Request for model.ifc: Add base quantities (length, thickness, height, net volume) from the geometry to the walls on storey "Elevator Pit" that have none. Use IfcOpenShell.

First a look at what the model holds.

```python
import ifcopenshell
import ifcopenshell.util.element
import ifcopenshell.util.unit

model = ifcopenshell.open("model.ifc")
print(model.schema)
for unit_type in ("LENGTHUNIT", "AREAUNIT", "VOLUMEUNIT"):
    print(unit_type, ifcopenshell.util.unit.calculate_unit_scale(model, unit_type))
storey = next(s for s in model.by_type("IfcBuildingStorey") if s.Name == "Elevator Pit")
walls = [e for e in ifcopenshell.util.element.get_decomposition(storey) if e.is_a("IfcWall")]
for e in sorted(walls, key=lambda e: e.id()):
    print(e.id(), e.is_a(), e.Name, list(ifcopenshell.util.element.get_psets(e, qtos_only=True)), sep=" | ")
```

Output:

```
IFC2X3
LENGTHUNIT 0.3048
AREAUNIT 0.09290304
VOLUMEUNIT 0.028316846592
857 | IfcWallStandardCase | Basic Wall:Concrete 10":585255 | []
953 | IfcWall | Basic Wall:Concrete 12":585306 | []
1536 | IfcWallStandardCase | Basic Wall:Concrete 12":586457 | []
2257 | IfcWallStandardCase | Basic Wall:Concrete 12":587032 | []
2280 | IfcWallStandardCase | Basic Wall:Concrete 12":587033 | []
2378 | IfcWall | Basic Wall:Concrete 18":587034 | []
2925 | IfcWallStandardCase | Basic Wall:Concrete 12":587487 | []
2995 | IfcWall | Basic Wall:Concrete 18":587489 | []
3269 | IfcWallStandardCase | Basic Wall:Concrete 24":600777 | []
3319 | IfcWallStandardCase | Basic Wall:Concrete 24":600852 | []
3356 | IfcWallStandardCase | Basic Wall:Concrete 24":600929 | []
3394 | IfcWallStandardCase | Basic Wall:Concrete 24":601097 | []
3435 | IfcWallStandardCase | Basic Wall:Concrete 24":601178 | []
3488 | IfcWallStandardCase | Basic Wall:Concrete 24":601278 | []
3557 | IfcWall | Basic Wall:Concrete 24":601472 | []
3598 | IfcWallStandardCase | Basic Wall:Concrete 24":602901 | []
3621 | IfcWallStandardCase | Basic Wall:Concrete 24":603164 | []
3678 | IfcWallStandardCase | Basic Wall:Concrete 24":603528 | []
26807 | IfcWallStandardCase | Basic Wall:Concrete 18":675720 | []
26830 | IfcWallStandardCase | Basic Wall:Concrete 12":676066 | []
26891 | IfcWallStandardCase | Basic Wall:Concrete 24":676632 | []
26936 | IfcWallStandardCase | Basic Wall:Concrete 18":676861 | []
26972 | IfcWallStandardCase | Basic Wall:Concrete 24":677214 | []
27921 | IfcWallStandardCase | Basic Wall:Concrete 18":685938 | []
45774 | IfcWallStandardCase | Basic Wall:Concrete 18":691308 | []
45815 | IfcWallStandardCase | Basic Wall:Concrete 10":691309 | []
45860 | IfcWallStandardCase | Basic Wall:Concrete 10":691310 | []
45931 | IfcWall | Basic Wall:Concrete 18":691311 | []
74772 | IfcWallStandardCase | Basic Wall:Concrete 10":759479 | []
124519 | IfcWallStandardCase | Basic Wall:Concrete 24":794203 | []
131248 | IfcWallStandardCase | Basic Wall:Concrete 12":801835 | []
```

```python
import ifcopenshell
import ifcopenshell.api.pset
import ifcopenshell.geom
import ifcopenshell.util.element
import ifcopenshell.util.shape
import ifcopenshell.util.unit

model = ifcopenshell.open("model.ifc")
unit_scale = ifcopenshell.util.unit.calculate_unit_scale(model)
volume_scale = ifcopenshell.util.unit.calculate_unit_scale(model, "VOLUMEUNIT")
settings = ifcopenshell.geom.settings()

storey = next(s for s in model.by_type("IfcBuildingStorey") if s.Name == "Elevator Pit")
walls = [e for e in ifcopenshell.util.element.get_decomposition(storey) if e.is_a("IfcWall")]

for e in sorted(walls, key=lambda e: e.id()):
    if ifcopenshell.util.element.get_psets(e, qtos_only=True, should_inherit=False):
        continue
    # Geometry comes back in metres, in the element's own axes.
    shape = ifcopenshell.geom.create_shape(settings, e)
    values = {
        "Length": ifcopenshell.util.shape.get_x(shape.geometry) / unit_scale,
        "Width": ifcopenshell.util.shape.get_y(shape.geometry) / unit_scale,
        "Height": ifcopenshell.util.shape.get_z(shape.geometry) / unit_scale,
        "NetVolume": ifcopenshell.util.shape.get_volume(shape.geometry) / volume_scale,
    }
    qto = ifcopenshell.api.pset.add_qto(model, product=e, name="BaseQuantities")
    ifcopenshell.api.pset.edit_qto(model, qto=qto, properties=values)
    print(e.id(), {k: round(v, 3) for k, v in values.items()})

model.write("model_edited.ifc")
```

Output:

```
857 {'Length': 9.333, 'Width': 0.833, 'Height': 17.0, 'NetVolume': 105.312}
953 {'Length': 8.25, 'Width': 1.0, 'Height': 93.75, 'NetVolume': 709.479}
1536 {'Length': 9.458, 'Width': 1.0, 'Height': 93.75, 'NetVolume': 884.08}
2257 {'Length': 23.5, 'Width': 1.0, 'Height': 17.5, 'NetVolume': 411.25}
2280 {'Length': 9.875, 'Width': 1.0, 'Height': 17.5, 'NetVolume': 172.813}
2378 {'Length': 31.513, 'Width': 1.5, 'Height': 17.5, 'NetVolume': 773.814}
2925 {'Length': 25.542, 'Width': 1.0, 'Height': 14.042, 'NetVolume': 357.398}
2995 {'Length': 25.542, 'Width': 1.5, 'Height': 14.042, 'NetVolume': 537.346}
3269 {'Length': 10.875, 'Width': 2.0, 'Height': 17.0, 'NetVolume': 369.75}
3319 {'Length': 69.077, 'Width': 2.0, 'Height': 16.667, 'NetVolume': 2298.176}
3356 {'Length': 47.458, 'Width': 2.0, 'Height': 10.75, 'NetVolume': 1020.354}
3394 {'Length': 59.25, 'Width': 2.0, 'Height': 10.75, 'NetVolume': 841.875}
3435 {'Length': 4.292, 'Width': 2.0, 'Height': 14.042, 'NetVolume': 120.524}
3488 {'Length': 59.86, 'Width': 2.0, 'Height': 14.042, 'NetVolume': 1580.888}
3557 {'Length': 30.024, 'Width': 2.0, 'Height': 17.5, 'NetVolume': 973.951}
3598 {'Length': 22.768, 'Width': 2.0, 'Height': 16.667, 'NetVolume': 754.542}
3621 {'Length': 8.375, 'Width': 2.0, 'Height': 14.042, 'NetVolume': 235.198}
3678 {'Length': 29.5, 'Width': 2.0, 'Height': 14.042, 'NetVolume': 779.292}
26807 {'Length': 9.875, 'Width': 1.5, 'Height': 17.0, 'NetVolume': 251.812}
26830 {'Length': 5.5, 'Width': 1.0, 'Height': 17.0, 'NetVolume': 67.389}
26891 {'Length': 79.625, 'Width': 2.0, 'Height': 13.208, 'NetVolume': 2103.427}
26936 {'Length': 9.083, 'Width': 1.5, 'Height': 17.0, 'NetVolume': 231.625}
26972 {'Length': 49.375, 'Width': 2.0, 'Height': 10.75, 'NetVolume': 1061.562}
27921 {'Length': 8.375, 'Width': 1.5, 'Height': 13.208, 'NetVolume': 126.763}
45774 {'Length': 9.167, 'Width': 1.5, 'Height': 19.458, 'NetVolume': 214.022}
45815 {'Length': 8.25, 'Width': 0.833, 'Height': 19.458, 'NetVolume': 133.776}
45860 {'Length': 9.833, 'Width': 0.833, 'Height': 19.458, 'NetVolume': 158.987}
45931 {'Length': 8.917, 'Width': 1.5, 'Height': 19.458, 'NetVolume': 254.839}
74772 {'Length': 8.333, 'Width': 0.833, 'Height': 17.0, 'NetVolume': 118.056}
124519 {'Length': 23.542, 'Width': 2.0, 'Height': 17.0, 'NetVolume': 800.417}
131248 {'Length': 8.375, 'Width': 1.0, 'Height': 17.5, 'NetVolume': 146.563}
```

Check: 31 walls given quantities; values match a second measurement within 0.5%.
